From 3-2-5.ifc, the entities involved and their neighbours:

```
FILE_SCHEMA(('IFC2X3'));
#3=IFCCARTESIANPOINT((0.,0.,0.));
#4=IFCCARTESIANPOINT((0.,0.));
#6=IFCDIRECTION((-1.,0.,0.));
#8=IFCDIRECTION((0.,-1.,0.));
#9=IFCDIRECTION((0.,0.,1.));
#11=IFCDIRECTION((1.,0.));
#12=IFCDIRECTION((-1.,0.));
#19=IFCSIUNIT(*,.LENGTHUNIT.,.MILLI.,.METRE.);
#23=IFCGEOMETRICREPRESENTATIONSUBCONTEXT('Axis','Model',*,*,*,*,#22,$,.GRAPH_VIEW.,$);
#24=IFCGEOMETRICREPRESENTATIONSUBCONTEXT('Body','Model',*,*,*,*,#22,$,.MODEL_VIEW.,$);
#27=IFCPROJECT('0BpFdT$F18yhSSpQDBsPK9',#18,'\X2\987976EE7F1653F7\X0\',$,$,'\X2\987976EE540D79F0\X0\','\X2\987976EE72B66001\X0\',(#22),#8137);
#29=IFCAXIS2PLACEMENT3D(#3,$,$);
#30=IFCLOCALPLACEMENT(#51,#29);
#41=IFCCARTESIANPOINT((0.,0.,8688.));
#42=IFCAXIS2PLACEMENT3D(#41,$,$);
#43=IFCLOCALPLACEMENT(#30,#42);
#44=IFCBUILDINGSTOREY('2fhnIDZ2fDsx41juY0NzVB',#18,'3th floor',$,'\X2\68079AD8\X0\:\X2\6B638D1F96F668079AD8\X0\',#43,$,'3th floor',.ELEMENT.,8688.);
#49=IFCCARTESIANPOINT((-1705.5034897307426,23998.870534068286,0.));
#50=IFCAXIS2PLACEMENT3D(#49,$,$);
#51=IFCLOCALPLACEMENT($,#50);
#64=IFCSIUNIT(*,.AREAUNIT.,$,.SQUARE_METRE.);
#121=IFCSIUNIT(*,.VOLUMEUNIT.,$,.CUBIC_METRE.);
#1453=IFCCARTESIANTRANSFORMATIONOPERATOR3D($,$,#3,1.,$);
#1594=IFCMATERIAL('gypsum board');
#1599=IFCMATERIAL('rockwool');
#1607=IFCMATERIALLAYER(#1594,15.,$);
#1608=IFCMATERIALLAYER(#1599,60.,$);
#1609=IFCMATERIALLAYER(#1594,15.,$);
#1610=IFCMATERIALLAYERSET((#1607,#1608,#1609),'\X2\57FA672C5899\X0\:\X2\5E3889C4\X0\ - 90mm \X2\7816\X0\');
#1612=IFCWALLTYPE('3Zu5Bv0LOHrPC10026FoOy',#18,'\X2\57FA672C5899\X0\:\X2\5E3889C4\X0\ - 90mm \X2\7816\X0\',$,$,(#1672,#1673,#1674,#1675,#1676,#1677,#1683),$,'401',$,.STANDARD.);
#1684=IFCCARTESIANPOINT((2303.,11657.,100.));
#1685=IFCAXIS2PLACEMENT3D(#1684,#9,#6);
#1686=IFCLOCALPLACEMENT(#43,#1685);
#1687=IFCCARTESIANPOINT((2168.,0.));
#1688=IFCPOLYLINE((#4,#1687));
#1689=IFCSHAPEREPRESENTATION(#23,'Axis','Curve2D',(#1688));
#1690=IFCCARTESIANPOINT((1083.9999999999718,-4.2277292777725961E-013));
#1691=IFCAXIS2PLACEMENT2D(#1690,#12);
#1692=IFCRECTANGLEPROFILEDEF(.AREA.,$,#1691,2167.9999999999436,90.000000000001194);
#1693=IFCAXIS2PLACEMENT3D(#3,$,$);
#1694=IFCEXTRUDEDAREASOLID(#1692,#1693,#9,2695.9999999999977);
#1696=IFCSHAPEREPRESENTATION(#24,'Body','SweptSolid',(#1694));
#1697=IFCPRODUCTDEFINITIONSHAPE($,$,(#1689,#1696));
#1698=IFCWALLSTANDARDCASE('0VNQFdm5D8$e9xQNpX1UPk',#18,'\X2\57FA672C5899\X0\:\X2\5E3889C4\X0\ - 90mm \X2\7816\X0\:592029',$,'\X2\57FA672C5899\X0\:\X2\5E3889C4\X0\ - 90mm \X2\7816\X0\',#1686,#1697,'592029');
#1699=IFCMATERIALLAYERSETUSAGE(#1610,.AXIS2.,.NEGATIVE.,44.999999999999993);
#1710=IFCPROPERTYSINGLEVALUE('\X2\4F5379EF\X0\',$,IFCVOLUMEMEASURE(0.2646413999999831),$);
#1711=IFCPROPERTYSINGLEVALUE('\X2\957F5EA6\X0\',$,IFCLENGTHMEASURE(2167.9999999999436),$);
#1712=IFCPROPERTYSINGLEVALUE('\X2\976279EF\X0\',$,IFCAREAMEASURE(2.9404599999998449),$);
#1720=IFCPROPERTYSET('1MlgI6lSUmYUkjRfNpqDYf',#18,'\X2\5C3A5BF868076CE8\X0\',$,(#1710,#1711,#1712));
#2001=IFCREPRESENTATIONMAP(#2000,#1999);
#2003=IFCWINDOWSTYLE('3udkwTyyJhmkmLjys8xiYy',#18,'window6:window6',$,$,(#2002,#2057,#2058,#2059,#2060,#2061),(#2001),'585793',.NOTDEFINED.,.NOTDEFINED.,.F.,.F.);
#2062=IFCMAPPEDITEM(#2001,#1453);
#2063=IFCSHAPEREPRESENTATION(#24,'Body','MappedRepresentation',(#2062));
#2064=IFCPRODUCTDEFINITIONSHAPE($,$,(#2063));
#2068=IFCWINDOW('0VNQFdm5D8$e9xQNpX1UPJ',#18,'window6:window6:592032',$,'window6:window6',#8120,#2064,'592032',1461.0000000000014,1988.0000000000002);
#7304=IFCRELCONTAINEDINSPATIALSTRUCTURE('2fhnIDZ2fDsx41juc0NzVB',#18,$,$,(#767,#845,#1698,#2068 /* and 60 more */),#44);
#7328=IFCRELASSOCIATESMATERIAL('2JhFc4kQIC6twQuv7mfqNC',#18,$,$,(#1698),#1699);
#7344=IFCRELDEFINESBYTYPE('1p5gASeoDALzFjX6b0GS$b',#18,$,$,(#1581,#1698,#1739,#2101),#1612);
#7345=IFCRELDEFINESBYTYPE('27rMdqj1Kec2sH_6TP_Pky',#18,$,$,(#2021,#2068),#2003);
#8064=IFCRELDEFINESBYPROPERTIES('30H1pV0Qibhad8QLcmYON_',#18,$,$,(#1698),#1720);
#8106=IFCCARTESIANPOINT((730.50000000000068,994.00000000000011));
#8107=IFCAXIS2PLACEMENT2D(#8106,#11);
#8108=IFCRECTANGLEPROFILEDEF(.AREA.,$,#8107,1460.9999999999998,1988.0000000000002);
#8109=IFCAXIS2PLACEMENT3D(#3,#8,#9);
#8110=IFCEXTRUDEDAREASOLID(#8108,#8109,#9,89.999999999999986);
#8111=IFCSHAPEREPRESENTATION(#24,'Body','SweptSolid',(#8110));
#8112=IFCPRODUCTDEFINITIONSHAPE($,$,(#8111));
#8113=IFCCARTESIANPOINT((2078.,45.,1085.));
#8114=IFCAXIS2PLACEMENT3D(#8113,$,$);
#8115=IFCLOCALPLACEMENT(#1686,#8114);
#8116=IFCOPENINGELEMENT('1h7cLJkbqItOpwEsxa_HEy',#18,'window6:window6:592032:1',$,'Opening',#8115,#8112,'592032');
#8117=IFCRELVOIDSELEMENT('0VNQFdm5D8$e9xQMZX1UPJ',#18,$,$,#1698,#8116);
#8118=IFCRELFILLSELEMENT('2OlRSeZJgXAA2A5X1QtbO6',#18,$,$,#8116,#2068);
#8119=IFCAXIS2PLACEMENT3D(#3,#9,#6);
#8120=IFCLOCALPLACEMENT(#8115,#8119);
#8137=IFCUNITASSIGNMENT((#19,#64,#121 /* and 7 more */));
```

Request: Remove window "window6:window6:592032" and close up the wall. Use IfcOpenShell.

```python
import ifcopenshell
import ifcopenshell.api.feature
import ifcopenshell.api.pset
import ifcopenshell.api.root
import ifcopenshell.geom
import ifcopenshell.util.element
import ifcopenshell.util.shape
import ifcopenshell.util.unit

model = ifcopenshell.open("3-2-5.ifc")
area_scale = ifcopenshell.util.unit.calculate_unit_scale(model, "AREAUNIT")
volume_scale = ifcopenshell.util.unit.calculate_unit_scale(model, "VOLUMEUNIT")
settings = ifcopenshell.geom.settings()


def volume(element):
    """Net volume in cubic metres, openings subtracted."""
    shape = ifcopenshell.geom.create_shape(settings, element)
    return ifcopenshell.util.shape.get_volume(shape.geometry)


window = model.by_guid("0VNQFdm5D8$e9xQNpX1UPJ")
opening = window.FillsVoids[0].RelatingOpeningElement
wall = opening.VoidsElements[0].RelatingBuildingElement
before = volume(wall)

ifcopenshell.api.root.remove_product(model, product=window)
ifcopenshell.api.feature.remove_feature(model, feature=opening)

after = volume(wall)
thickness = 0.09  # wall thickness in metres

# Update the wall's stored quantities.
pset = model.by_id(ifcopenshell.util.element.get_pset(wall, "尺寸标注", should_inherit=False)["id"])
ifcopenshell.api.pset.edit_pset(model, pset=pset, properties={
    "体积": model.create_entity("IfcVolumeMeasure", after / volume_scale),
    "面积": model.create_entity("IfcAreaMeasure", after / thickness / area_scale),
})

print(f"wall volume {before:.3f} -> {after:.3f} m3")

model.write("3-2-5_edited.ifc")
```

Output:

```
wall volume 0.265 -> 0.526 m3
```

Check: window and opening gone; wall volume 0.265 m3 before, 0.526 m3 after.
